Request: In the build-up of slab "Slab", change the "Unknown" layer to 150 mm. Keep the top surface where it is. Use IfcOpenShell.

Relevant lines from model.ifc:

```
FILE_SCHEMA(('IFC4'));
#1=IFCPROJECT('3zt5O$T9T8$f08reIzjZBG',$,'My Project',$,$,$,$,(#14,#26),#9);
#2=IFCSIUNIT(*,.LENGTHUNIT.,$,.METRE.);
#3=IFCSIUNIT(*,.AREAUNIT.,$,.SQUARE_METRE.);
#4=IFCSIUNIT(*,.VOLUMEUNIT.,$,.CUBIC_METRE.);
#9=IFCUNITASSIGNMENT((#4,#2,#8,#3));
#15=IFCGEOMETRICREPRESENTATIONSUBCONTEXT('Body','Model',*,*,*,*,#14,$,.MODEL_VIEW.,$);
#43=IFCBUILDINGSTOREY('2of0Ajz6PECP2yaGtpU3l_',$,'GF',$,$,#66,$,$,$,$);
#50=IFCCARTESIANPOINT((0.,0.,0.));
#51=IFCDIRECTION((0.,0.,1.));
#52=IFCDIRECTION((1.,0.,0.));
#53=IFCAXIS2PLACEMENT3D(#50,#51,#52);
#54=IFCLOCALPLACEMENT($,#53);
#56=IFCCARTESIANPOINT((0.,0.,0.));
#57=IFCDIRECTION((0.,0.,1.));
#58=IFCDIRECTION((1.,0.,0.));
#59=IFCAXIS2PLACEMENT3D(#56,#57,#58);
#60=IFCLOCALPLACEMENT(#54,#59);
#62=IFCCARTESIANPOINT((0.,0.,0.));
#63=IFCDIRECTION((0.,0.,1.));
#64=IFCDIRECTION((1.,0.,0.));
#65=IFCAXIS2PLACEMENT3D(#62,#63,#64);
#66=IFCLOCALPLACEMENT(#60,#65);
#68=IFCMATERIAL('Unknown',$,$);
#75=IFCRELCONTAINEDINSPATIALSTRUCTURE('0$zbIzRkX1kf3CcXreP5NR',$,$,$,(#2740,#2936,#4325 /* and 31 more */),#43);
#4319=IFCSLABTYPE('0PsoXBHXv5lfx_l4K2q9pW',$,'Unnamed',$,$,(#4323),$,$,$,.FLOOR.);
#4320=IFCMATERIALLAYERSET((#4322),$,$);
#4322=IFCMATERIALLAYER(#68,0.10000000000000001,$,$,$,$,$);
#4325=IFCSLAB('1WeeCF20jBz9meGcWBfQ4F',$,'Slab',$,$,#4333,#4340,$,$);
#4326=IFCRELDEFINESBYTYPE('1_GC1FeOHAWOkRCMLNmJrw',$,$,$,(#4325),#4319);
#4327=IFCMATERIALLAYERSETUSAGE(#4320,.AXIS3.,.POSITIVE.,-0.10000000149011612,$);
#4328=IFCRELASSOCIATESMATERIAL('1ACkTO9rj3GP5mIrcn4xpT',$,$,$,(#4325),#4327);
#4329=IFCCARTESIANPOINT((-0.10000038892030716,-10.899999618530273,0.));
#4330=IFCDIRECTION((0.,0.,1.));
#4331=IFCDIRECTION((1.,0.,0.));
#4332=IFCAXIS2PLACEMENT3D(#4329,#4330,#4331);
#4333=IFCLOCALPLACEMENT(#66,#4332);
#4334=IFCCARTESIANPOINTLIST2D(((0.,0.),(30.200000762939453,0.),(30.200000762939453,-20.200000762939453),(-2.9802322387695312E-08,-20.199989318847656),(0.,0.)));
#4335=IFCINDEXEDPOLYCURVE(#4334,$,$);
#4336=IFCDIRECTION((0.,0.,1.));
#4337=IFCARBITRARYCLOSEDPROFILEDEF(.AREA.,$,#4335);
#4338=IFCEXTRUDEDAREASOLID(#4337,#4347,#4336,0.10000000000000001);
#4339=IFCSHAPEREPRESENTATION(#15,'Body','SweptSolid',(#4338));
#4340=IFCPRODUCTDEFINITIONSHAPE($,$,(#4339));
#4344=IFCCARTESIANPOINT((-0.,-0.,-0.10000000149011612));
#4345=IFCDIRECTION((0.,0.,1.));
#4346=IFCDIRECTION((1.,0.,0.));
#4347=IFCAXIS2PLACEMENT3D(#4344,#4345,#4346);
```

```python
import ifcopenshell
import ifcopenshell.util.element
import ifcopenshell.util.representation
import ifcopenshell.util.unit

model = ifcopenshell.open("model.ifc")
unit_scale = ifcopenshell.util.unit.calculate_unit_scale(model)

layer_set = model.by_id(4320)
layer = next(l for l in layer_set.MaterialLayers if l.Material and l.Material.Name == "Unknown")
change = 0.15 / unit_scale - layer.LayerThickness
layer.LayerThickness += change

# Geometry does not follow the layer set by itself.
slabs = [e for e in ifcopenshell.util.element.get_elements_by_material(model, layer_set) if e.is_a("IfcSlab")]
for slab in sorted(slabs, key=lambda e: e.id()):
    body = ifcopenshell.util.representation.get_representation(slab, "Model", "Body")
    solid = body.Items[0]
    old_depth = solid.Depth
    solid.Depth += change
    # Extruded upwards: lower the start of the extrusion so the top stays.
    x, y, z = solid.Position.Location.Coordinates
    solid.Position.Location = model.createIfcCartesianPoint((x, y, z - change))
    print(slab.id(), f"{old_depth:g} -> {solid.Depth:g}")

# The layers are counted up from the underside, which has moved.
for usage in {ifcopenshell.util.element.get_material(slab) for slab in slabs}:
    usage.OffsetFromReferenceLine -= change

model.write("model_rev.ifc")
```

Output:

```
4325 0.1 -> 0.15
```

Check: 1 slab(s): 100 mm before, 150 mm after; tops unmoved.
